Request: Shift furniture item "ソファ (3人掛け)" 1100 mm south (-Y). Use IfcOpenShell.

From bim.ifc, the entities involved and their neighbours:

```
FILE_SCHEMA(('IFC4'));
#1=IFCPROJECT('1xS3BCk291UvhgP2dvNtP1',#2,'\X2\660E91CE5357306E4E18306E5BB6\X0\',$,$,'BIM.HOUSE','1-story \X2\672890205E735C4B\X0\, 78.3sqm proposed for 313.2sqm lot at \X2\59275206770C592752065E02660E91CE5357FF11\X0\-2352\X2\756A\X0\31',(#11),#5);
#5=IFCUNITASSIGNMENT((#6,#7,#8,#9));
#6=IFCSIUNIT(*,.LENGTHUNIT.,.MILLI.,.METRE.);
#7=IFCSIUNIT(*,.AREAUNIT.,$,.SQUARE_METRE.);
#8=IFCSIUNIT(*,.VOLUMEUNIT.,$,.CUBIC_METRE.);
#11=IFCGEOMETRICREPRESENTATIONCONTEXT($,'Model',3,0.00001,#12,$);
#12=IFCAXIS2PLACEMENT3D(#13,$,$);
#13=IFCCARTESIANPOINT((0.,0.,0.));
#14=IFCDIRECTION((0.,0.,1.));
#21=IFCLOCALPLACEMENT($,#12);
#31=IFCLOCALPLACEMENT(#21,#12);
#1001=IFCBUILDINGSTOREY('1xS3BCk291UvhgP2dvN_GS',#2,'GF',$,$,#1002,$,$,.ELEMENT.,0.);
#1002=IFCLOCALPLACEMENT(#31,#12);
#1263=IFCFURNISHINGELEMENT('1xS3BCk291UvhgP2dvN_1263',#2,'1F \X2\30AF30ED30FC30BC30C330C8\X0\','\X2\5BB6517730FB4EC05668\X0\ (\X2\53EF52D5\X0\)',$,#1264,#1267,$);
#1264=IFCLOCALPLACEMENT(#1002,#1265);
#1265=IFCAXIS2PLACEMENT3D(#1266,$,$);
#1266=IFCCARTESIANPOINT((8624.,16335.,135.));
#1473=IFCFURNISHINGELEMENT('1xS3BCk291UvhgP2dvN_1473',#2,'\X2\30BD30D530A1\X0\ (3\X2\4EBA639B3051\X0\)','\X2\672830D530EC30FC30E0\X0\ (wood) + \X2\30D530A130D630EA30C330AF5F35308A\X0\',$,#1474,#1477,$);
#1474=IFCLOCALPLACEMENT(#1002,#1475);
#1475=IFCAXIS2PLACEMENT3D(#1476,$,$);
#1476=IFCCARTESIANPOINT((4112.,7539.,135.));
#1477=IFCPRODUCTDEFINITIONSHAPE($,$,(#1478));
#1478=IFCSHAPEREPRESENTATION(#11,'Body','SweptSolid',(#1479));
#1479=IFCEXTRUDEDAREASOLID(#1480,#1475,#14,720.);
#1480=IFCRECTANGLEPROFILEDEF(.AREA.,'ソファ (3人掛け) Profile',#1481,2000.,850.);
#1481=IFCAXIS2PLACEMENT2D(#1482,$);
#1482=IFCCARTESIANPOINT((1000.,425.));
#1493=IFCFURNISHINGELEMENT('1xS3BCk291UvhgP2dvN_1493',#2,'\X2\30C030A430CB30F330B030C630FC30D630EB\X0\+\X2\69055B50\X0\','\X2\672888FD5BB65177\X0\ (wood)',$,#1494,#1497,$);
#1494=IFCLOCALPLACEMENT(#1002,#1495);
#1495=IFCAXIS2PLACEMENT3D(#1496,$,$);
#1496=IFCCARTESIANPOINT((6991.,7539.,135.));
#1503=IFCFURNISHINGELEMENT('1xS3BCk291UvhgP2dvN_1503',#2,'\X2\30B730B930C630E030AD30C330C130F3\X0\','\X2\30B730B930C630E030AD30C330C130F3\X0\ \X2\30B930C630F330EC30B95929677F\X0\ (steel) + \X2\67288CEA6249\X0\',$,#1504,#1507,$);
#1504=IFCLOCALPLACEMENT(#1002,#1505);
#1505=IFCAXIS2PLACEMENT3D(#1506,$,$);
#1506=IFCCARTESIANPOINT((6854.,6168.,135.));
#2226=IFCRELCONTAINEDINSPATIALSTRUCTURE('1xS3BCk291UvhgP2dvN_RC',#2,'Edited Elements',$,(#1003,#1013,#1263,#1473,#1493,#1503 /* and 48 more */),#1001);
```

```python
import ifcopenshell
import ifcopenshell.api.geometry
import ifcopenshell.util.placement

model = ifcopenshell.open("bim.ifc")

item = model.by_guid("1xS3BCk291UvhgP2dvN_1473")
matrix = ifcopenshell.util.placement.get_local_placement(item.ObjectPlacement)
matrix[1, 3] -= 1100.0
ifcopenshell.api.geometry.edit_object_placement(model, product=item, matrix=matrix, is_si=False)

print(ifcopenshell.util.placement.get_local_placement(item.ObjectPlacement).round(3) + 0.0)

model.write("bim_rev.ifc")
```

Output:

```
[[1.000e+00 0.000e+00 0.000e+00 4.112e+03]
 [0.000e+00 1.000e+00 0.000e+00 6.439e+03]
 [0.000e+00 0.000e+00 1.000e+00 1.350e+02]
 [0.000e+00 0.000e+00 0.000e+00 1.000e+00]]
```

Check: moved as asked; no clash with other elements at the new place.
